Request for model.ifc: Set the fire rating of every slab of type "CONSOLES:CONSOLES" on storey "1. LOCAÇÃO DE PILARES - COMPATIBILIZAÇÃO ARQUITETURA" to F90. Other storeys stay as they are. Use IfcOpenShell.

First a look at what the model holds.

```python
import ifcopenshell
import ifcopenshell.util.element

model = ifcopenshell.open("model.ifc")
print(model.schema)
storey = next(s for s in model.by_type("IfcBuildingStorey") if s.Name == "1. LOCAÇÃO DE PILARES - COMPATIBILIZAÇÃO ARQUITETURA")
slabs = [e for e in ifcopenshell.util.element.get_decomposition(storey) if e.is_a("IfcSlab")]
seen = {}
for e in slabs:
    element_type = ifcopenshell.util.element.get_type(e)
    key = (element_type.Name if element_type != e and element_type else None, ifcopenshell.util.element.get_pset(e, "Pset_SlabCommon", "FireRating"))
    seen[key] = seen.get(key, 0) + 1
for (name, value), count in sorted(seen.items(), key=str):
    print(count, "x", name, "|", value)
```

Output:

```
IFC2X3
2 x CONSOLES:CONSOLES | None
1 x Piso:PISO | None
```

```python
import ifcopenshell
import ifcopenshell.api.pset
import ifcopenshell.util.element

model = ifcopenshell.open("model.ifc")

storey = next(s for s in model.by_type("IfcBuildingStorey") if s.Name == "1. LOCAÇÃO DE PILARES - COMPATIBILIZAÇÃO ARQUITETURA")
slabs = [e for e in ifcopenshell.util.element.get_decomposition(storey) if e.is_a("IfcSlab")]

count = 0
for e in slabs:
    element_type = ifcopenshell.util.element.get_type(e)
    if element_type in (None, e) or element_type.Name != "CONSOLES:CONSOLES":
        continue
    # add_pset returns the element's existing set when there is one.
    pset = ifcopenshell.api.pset.add_pset(model, product=e, name="Pset_SlabCommon")
    ifcopenshell.api.pset.edit_pset(model, pset=pset, properties={"FireRating": "F90"})
    count += 1

print(count, "slabs updated")

model.write("model-out.ifc")
```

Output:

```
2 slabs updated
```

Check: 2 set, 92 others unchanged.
